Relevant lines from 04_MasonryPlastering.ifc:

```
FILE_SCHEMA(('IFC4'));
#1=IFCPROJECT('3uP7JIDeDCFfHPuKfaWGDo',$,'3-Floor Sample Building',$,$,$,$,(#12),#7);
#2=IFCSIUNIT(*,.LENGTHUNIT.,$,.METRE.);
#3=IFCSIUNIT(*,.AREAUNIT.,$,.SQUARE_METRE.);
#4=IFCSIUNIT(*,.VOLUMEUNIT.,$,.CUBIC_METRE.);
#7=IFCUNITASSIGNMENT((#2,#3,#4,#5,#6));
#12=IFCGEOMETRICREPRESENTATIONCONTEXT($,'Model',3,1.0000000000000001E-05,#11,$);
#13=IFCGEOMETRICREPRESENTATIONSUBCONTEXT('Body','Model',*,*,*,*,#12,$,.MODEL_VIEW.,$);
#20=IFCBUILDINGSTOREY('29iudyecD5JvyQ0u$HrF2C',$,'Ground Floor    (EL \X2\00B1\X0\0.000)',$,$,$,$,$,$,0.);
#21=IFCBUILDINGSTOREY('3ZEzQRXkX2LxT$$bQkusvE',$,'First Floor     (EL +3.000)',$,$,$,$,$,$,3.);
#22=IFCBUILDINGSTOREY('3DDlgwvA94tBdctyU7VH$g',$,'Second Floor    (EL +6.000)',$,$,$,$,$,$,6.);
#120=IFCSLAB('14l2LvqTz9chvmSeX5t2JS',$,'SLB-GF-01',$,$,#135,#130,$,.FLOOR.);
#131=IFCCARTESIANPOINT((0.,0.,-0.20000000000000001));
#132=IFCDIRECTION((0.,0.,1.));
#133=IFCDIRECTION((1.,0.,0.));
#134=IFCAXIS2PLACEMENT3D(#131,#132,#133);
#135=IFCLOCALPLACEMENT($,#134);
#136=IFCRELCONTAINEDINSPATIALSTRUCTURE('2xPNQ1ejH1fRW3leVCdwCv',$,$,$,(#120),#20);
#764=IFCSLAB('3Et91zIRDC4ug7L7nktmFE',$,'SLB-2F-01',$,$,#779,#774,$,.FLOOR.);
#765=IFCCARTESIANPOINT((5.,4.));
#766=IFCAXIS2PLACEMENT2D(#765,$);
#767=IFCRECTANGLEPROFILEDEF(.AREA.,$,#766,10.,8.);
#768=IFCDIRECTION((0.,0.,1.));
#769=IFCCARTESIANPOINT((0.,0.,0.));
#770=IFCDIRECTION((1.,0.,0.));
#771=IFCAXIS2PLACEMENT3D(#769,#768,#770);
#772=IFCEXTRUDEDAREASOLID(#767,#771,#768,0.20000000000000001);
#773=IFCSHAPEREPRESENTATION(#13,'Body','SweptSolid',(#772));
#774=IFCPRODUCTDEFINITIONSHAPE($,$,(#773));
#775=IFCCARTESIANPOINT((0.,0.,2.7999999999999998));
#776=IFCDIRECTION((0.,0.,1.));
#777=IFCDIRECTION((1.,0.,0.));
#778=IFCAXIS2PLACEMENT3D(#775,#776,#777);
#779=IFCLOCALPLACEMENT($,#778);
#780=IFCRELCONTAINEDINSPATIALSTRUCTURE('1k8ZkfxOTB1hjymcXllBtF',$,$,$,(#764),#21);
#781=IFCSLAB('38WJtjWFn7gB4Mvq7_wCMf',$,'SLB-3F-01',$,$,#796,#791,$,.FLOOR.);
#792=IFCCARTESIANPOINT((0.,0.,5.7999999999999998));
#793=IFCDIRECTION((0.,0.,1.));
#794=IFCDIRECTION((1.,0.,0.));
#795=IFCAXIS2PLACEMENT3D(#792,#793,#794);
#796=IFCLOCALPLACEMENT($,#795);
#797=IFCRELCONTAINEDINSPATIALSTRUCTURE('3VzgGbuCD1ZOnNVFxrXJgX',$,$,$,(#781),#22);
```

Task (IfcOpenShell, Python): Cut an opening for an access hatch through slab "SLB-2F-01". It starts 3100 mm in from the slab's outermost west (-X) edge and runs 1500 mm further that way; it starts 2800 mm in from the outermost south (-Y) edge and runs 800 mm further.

```python
import numpy as np
import ifcopenshell
import ifcopenshell.api.feature
import ifcopenshell.api.geometry
import ifcopenshell.api.root
import ifcopenshell.geom
import ifcopenshell.util.placement
import ifcopenshell.util.representation
import ifcopenshell.util.shape
import ifcopenshell.util.unit

model = ifcopenshell.open("04_MasonryPlastering.ifc")
unit_scale = ifcopenshell.util.unit.calculate_unit_scale(model)
settings = ifcopenshell.geom.settings()


def volume(element):
    """Net volume in cubic metres, openings subtracted."""
    shape = ifcopenshell.geom.create_shape(settings, element)
    return ifcopenshell.util.shape.get_volume(shape.geometry)


slab = model.by_guid("3Et91zIRDC4ug7L7nktmFE")
before = volume(slab)

# Extent in the slab's own axes, in metres. The edges named are its -X and -Y sides.
slab_shape = ifcopenshell.geom.create_shape(settings, slab)
vertices = ifcopenshell.util.shape.get_vertices(slab_shape.geometry)
x_min, y_min, bottom = vertices.min(axis=0)
top = vertices[:, 2].max()

opening = ifcopenshell.api.root.create_entity(model, ifc_class="IfcOpeningElement", name="Access hatch opening", predefined_type="OPENING")
context = ifcopenshell.util.representation.get_context(model, "Model", "Body", "MODEL_VIEW")
width, depth = 1.5, 0.8
outline = [(0.0, 0.0), (width, 0.0), (width, depth), (0.0, depth), (0.0, 0.0)]
# Overshoot both faces by 50 mm so the cut is clean.
shape = ifcopenshell.api.geometry.add_slab_representation(
    model, context=context, depth=top - bottom + 0.1, polyline=outline
)
ifcopenshell.api.geometry.assign_representation(model, product=opening, representation=shape)

matrix = ifcopenshell.util.placement.get_local_placement(slab.ObjectPlacement)
matrix[:, 3] = matrix @ np.append(np.array([x_min + 3.1, y_min + 2.8, bottom - 0.05]) / unit_scale, 1.0)
ifcopenshell.api.geometry.edit_object_placement(model, product=opening, matrix=matrix, is_si=False)
ifcopenshell.api.feature.add_feature(model, feature=opening, element=slab)

after = volume(slab)

print(f"slab volume {before:.3f} -> {after:.3f} m3")

model.write("04_MasonryPlastering_v2.ifc")
```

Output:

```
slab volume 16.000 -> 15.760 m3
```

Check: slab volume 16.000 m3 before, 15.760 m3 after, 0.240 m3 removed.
